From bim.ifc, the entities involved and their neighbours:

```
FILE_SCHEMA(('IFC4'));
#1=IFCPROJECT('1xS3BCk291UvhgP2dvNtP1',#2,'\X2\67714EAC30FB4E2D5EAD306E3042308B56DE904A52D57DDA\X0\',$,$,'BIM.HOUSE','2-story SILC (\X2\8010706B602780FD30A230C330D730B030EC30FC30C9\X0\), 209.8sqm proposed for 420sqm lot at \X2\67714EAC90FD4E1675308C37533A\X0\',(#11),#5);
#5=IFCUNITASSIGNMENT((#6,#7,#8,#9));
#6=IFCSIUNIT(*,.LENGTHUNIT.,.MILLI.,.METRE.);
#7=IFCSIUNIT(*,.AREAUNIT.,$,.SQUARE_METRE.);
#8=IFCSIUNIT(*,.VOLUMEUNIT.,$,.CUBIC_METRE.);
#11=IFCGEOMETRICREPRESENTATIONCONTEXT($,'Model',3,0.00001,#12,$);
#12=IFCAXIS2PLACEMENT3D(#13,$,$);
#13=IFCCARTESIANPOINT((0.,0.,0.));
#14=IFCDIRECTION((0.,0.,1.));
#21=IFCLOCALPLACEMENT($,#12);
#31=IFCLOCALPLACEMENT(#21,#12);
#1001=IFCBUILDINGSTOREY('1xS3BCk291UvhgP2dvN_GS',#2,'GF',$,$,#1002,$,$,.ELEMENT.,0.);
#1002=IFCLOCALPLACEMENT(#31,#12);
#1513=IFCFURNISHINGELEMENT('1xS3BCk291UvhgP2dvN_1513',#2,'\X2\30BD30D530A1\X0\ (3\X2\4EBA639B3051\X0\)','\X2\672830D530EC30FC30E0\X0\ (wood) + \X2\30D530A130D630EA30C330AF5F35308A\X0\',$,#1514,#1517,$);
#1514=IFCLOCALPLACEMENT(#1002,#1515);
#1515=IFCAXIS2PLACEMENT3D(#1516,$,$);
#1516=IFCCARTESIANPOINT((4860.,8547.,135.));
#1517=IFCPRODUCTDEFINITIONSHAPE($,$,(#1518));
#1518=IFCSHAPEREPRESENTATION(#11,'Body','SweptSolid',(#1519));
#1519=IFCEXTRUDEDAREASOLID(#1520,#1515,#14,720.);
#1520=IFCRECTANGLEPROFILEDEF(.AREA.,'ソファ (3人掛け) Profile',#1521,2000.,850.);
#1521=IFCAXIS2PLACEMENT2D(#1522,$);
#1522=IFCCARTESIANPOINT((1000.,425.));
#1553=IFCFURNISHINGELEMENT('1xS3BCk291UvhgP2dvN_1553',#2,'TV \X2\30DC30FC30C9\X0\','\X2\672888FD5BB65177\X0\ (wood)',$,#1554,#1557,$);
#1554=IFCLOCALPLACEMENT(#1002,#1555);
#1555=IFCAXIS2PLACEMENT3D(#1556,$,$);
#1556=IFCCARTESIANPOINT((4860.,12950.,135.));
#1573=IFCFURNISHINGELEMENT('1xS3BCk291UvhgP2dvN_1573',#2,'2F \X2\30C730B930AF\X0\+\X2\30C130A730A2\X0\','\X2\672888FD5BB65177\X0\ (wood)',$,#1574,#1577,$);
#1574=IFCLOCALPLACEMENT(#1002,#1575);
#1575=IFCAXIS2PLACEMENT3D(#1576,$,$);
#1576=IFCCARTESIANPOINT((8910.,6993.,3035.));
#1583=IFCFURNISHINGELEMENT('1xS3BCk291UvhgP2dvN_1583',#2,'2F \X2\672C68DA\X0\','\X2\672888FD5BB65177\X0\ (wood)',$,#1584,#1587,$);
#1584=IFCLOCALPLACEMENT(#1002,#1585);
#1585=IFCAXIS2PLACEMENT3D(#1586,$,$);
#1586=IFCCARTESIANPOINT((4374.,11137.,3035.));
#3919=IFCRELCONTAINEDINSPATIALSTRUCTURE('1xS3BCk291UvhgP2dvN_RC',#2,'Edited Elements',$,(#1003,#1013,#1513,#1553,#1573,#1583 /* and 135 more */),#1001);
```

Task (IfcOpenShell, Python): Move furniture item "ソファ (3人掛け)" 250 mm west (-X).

```python
import ifcopenshell
import ifcopenshell.api.geometry
import ifcopenshell.util.placement
import ifcopenshell.util.unit

model = ifcopenshell.open("bim.ifc")
unit_scale = ifcopenshell.util.unit.calculate_unit_scale(model)

item = model.by_guid("1xS3BCk291UvhgP2dvN_1513")
matrix = ifcopenshell.util.placement.get_local_placement(item.ObjectPlacement)
matrix[0, 3] -= 0.25 / unit_scale
ifcopenshell.api.geometry.edit_object_placement(model, product=item, matrix=matrix, is_si=False)

print(ifcopenshell.util.placement.get_local_placement(item.ObjectPlacement).round(3) + 0.0)

model.write("bim_updated.ifc")
```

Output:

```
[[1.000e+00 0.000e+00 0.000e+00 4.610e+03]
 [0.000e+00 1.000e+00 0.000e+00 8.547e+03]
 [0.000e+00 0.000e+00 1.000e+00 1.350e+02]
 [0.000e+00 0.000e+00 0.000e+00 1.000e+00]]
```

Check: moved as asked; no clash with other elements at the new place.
